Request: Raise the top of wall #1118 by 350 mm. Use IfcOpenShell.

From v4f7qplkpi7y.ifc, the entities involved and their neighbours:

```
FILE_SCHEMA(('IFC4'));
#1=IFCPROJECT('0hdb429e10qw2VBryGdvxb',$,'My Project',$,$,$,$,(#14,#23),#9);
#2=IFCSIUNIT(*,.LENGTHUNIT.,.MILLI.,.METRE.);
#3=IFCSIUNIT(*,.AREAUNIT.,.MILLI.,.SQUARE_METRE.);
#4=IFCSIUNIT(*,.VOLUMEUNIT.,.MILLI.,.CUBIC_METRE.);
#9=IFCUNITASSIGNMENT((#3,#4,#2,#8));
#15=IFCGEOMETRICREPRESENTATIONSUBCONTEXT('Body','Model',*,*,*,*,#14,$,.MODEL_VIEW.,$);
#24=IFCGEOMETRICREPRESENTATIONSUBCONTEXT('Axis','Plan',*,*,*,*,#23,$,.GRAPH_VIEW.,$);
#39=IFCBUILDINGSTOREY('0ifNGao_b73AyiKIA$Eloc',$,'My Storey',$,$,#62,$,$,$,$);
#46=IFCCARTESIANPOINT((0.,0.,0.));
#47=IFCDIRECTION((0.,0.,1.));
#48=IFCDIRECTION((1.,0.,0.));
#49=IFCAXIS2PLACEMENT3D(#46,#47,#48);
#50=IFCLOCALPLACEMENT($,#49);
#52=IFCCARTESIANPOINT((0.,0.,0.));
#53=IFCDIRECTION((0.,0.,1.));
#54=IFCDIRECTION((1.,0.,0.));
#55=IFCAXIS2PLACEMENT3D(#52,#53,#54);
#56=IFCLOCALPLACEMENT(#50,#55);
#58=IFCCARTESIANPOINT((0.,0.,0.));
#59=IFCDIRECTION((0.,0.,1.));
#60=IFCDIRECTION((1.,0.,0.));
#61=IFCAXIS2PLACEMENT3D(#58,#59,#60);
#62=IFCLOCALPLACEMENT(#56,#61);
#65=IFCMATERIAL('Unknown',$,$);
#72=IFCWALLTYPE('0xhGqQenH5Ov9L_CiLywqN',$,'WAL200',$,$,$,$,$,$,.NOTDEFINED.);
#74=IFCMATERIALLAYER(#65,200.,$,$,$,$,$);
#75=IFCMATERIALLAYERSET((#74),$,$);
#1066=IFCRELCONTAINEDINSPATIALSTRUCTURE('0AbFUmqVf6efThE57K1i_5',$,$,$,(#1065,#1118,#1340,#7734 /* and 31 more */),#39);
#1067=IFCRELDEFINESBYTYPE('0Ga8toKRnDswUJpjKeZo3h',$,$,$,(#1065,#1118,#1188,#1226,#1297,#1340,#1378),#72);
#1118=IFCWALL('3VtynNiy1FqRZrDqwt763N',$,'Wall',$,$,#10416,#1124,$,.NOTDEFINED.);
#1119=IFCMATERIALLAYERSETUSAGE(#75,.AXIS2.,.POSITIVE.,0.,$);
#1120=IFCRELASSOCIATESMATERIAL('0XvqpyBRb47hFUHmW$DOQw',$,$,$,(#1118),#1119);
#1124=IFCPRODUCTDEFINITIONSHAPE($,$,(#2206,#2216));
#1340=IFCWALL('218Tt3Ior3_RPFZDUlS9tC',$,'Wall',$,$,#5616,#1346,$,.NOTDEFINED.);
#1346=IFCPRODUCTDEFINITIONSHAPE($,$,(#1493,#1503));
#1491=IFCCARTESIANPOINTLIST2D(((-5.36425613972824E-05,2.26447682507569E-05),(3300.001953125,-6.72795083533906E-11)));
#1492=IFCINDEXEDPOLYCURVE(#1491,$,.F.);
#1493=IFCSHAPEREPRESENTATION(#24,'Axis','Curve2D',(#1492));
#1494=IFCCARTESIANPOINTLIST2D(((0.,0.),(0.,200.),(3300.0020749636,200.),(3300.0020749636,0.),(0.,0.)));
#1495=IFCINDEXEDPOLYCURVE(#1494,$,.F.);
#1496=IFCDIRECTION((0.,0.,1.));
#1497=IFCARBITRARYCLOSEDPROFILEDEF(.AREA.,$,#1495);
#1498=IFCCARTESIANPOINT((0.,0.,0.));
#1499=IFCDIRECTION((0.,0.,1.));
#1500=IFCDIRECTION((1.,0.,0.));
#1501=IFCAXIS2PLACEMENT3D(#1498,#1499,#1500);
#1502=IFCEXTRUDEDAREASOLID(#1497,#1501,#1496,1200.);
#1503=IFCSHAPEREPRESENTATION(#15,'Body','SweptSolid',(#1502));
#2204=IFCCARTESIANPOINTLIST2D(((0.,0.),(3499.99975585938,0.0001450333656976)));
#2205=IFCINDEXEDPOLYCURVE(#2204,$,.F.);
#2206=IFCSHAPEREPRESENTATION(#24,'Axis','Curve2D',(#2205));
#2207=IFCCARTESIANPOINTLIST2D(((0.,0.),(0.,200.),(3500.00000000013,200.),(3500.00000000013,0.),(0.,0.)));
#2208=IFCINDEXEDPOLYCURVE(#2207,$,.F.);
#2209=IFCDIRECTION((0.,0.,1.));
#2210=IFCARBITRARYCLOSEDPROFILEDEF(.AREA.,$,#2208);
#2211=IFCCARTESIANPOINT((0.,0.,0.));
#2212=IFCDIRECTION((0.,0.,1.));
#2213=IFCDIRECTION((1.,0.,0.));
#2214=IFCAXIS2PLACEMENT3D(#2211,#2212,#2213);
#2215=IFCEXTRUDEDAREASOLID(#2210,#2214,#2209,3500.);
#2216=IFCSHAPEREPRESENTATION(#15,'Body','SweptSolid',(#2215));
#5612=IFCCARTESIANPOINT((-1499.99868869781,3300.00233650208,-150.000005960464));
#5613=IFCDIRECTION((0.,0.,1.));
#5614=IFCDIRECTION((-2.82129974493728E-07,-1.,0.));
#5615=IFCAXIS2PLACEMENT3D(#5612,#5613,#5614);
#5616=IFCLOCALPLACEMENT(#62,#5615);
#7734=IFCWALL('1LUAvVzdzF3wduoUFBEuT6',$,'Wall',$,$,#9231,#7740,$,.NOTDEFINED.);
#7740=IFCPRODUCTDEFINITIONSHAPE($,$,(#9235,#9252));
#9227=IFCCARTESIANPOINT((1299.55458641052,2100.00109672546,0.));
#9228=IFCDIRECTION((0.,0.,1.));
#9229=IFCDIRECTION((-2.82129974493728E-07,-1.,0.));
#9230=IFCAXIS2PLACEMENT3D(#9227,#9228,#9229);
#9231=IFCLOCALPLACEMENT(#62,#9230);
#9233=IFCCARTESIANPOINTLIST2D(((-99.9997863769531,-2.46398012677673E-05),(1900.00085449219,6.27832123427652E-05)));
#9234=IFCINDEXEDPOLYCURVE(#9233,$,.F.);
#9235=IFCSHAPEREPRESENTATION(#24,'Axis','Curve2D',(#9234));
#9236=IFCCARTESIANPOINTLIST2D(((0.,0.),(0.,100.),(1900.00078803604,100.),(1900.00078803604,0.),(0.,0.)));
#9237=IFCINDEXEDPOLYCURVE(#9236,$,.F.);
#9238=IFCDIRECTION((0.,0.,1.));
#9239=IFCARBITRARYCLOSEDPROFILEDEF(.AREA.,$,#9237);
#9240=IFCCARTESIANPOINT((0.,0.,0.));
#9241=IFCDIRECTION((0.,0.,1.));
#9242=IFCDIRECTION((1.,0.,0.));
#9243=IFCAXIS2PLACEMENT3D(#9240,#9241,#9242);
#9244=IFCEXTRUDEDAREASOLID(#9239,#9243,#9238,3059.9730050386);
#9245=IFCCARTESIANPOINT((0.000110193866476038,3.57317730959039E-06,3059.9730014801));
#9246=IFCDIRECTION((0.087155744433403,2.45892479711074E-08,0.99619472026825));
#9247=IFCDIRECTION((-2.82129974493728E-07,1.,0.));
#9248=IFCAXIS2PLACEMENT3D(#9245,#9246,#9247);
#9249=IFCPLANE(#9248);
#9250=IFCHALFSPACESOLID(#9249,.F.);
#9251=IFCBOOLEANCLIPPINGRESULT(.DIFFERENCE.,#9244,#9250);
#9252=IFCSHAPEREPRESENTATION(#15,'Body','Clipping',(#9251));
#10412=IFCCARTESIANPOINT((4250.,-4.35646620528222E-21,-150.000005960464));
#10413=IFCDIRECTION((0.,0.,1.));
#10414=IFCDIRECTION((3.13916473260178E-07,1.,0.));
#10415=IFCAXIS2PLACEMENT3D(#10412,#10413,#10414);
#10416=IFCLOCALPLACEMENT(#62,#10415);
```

```python
import ifcopenshell
import ifcopenshell.geom
import ifcopenshell.util.representation
import ifcopenshell.util.shape
import ifcopenshell.util.unit

model = ifcopenshell.open("v4f7qplkpi7y.ifc")
unit_scale = ifcopenshell.util.unit.calculate_unit_scale(model)
settings = ifcopenshell.geom.settings()


def volume(element):
    """Net volume in cubic metres, openings subtracted."""
    shape = ifcopenshell.geom.create_shape(settings, element)
    return ifcopenshell.util.shape.get_volume(shape.geometry)


wall = model.by_guid("3VtynNiy1FqRZrDqwt763N")
before = volume(wall)

body = ifcopenshell.util.representation.get_representation(wall, "Model", "Body")
solid = body.Items[0]
old_height = solid.Depth
solid.Depth += 0.35 / unit_scale
after = volume(wall)

print(f"height {old_height:g} -> {solid.Depth:g}, volume {before:.3f} -> {after:.3f} m3")

model.write("v4f7qplkpi7y_edited.ifc")
```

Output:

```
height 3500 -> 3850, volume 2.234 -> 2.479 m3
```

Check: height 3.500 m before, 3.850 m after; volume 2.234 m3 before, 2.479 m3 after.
